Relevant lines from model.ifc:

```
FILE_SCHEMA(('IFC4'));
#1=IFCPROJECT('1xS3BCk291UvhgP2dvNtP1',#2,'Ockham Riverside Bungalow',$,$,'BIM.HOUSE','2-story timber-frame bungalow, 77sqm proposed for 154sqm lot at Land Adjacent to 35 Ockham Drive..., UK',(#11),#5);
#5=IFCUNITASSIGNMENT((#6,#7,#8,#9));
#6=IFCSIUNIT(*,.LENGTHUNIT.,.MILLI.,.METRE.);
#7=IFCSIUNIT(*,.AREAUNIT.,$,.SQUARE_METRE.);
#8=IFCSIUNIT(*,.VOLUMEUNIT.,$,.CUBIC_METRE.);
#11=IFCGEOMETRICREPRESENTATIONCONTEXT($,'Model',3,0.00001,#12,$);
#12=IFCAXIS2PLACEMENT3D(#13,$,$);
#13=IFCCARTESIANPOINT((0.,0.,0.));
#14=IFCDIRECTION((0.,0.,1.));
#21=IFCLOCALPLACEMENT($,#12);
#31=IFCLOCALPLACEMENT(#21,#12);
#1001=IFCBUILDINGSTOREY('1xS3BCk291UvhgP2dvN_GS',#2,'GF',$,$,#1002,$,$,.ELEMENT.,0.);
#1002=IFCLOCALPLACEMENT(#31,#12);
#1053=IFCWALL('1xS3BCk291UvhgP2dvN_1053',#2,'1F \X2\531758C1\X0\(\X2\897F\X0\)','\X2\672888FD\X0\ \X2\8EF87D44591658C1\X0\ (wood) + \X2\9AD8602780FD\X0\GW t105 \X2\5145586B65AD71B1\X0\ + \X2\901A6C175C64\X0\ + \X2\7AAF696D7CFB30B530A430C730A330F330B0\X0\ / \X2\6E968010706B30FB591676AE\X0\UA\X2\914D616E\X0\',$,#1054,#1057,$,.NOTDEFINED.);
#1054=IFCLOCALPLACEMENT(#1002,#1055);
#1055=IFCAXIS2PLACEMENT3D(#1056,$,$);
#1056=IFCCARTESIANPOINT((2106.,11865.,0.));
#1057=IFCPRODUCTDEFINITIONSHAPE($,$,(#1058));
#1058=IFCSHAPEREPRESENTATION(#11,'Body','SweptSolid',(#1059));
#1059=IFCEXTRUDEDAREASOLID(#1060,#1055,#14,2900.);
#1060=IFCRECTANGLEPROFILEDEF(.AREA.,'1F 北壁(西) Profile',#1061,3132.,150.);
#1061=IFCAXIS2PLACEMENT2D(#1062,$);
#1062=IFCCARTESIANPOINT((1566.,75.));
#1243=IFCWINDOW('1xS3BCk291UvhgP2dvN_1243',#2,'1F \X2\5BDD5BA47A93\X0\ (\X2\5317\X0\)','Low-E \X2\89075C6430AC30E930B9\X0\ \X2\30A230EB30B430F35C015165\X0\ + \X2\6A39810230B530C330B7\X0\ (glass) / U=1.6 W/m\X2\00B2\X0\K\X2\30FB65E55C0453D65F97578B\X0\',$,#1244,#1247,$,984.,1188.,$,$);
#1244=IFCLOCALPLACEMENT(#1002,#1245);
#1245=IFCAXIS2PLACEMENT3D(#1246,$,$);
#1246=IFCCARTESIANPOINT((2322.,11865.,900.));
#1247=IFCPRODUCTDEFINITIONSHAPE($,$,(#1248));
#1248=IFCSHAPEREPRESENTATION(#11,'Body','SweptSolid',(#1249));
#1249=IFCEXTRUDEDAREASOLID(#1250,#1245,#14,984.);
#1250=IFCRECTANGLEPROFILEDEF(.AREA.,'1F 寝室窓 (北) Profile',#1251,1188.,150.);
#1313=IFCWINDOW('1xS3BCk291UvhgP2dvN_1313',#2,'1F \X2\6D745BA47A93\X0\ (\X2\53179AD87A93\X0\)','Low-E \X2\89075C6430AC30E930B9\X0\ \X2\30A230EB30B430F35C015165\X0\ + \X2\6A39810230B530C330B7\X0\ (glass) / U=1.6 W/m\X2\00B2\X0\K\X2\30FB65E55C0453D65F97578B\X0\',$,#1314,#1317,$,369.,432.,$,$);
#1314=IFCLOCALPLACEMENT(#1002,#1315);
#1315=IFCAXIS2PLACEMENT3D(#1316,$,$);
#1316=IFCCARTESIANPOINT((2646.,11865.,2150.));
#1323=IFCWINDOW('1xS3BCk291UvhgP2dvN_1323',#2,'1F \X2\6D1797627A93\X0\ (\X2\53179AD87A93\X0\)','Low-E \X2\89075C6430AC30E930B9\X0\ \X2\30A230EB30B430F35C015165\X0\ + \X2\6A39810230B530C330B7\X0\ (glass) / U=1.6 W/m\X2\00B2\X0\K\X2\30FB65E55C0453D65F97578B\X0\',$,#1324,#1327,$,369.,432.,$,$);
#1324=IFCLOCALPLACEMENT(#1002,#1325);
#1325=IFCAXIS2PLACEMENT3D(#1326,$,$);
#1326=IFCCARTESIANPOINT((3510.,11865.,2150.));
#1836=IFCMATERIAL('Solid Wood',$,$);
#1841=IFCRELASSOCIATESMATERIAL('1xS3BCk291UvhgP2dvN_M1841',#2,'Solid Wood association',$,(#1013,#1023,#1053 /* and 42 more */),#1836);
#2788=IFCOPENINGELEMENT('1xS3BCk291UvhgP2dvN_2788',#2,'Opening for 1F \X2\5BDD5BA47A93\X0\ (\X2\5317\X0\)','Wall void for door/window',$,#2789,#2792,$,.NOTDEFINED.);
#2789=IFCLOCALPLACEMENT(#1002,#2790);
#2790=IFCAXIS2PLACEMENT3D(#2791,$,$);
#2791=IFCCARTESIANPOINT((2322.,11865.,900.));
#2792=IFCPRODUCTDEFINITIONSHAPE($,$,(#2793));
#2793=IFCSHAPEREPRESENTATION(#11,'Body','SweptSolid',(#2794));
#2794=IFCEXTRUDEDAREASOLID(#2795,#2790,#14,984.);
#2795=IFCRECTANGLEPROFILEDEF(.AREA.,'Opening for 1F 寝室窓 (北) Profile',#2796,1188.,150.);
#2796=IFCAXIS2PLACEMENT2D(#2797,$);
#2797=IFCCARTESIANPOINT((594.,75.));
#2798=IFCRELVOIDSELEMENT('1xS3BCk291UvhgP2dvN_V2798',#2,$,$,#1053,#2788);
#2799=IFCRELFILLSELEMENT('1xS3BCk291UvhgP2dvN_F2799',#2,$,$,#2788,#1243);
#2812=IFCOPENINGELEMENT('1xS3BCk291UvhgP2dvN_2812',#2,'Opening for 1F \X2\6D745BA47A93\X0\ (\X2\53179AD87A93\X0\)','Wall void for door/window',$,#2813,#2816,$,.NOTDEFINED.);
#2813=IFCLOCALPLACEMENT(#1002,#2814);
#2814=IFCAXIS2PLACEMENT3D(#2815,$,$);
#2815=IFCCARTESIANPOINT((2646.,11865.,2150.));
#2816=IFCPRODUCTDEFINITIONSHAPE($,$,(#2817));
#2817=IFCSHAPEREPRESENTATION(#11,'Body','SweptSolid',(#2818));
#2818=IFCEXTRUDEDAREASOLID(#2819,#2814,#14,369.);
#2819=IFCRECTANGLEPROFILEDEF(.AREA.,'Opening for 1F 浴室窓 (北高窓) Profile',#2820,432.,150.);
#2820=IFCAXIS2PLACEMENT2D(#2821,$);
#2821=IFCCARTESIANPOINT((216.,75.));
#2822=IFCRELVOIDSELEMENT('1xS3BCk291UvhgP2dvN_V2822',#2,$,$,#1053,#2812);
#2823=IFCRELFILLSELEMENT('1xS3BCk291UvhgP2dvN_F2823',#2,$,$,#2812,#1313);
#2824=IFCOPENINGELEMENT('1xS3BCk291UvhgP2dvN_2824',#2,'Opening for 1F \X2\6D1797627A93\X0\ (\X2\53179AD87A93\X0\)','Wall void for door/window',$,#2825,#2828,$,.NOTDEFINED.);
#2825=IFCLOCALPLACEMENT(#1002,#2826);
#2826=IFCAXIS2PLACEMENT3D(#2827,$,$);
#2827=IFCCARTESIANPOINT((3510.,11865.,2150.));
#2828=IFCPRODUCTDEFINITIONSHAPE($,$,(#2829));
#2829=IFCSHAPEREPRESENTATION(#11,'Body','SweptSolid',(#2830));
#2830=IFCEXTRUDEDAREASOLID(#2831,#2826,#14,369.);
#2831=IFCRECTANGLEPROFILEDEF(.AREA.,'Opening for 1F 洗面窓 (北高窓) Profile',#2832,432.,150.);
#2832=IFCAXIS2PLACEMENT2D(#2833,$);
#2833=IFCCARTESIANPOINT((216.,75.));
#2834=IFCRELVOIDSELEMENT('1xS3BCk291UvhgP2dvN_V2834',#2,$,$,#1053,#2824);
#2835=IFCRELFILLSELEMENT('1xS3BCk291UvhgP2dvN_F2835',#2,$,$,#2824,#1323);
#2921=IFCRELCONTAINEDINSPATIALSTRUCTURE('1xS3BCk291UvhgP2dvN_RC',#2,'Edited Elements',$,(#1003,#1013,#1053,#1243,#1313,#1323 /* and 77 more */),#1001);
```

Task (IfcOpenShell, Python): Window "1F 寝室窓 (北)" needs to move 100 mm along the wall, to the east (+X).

```python
import ifcopenshell
import ifcopenshell.api.geometry
import ifcopenshell.util.placement
import ifcopenshell.util.unit

model = ifcopenshell.open("model.ifc")
unit_scale = ifcopenshell.util.unit.calculate_unit_scale(model)

window = model.by_guid("1xS3BCk291UvhgP2dvN_1243")
opening = window.FillsVoids[0].RelatingOpeningElement
wall = opening.VoidsElements[0].RelatingBuildingElement

wall_matrix = ifcopenshell.util.placement.get_local_placement(wall.ObjectPlacement)
shift = wall_matrix[:3, 0] * 0.1 / unit_scale
before = ifcopenshell.util.placement.get_local_placement(window.ObjectPlacement)[:3, 3].copy()

# The window is not placed relative to its opening, so move both.
for product in (opening, window):
    matrix = ifcopenshell.util.placement.get_local_placement(product.ObjectPlacement)
    matrix[:3, 3] += shift
    ifcopenshell.api.geometry.edit_object_placement(model, product=product, matrix=matrix, is_si=False)

after = ifcopenshell.util.placement.get_local_placement(window.ObjectPlacement)[:3, 3]
print("window moved by", (after - before).round(3) + 0.0)

model.write("model_v2.ifc")
```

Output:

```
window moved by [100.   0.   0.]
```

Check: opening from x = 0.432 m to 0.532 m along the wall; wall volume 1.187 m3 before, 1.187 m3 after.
